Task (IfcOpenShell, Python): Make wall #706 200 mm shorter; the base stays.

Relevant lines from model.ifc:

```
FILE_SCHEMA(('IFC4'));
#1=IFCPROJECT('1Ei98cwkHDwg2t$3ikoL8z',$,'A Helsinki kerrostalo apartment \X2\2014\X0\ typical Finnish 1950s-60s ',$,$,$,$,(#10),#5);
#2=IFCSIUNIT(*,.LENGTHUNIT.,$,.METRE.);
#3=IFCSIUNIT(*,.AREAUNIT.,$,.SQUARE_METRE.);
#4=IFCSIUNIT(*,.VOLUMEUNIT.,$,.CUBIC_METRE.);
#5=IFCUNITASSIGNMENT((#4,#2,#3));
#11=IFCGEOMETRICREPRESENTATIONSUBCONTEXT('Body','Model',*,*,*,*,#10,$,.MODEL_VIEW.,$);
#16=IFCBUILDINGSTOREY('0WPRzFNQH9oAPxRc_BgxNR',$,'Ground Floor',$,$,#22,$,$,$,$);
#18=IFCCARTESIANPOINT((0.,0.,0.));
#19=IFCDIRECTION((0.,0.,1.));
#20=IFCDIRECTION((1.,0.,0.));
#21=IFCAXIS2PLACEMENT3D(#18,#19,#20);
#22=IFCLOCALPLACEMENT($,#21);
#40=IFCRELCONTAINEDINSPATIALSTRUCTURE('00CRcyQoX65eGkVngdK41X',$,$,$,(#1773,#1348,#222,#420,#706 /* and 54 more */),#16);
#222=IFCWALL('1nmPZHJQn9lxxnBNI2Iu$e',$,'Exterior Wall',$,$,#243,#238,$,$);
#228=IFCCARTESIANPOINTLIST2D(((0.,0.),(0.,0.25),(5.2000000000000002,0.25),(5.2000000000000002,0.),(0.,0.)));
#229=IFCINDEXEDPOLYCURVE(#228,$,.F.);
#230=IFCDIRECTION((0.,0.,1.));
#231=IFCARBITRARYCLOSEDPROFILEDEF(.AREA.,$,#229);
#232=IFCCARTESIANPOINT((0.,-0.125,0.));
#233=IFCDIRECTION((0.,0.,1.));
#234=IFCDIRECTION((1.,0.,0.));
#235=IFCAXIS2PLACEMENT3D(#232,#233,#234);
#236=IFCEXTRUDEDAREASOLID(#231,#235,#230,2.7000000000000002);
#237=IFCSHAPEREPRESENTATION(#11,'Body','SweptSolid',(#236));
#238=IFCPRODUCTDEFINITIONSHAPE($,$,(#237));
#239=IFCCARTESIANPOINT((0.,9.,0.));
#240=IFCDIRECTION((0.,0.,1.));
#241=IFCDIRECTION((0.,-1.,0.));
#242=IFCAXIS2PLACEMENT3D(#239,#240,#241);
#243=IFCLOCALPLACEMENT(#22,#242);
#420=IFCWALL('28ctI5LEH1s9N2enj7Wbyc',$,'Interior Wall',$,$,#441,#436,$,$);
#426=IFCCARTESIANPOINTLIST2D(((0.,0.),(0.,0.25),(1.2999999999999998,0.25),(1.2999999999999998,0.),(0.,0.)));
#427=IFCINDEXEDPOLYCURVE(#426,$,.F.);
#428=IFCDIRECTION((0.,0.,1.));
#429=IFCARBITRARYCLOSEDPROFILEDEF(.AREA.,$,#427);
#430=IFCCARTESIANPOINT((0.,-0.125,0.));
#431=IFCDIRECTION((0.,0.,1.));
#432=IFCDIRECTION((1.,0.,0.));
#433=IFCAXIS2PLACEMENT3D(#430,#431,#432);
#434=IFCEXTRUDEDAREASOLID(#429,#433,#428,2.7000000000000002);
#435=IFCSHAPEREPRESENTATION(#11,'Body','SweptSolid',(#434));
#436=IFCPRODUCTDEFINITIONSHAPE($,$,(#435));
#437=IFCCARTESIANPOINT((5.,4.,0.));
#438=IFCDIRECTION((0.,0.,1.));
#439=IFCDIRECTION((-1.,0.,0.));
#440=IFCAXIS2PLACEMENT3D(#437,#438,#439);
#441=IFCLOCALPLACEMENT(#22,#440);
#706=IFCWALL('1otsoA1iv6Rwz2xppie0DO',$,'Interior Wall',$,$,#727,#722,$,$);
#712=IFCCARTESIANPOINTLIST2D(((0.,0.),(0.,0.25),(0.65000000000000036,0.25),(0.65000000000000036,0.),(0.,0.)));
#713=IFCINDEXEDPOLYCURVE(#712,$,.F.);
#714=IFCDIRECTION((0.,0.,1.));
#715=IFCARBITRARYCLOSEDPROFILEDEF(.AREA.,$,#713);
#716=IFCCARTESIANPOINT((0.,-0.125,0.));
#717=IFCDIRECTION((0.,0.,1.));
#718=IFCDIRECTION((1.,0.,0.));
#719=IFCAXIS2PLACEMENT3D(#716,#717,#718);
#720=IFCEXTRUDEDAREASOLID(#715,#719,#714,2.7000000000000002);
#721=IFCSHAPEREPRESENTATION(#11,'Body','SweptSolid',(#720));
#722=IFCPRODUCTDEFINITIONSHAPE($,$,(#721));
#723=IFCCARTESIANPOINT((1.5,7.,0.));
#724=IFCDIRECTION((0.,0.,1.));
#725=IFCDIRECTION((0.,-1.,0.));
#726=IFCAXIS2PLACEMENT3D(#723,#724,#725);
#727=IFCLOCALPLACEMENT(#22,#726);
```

```python
import ifcopenshell
import ifcopenshell.geom
import ifcopenshell.util.representation
import ifcopenshell.util.shape

model = ifcopenshell.open("model.ifc")
settings = ifcopenshell.geom.settings()


def volume(element):
    """Net volume in cubic metres, openings subtracted."""
    shape = ifcopenshell.geom.create_shape(settings, element)
    return ifcopenshell.util.shape.get_volume(shape.geometry)


wall = model.by_id(706)
before = volume(wall)

body = ifcopenshell.util.representation.get_representation(wall, "Model", "Body")
solid = body.Items[0]
old_height = solid.Depth
solid.Depth -= 0.2
after = volume(wall)

print(f"height {old_height:g} -> {solid.Depth:g}, volume {before:.3f} -> {after:.3f} m3")

model.write("model_v2.ifc")
```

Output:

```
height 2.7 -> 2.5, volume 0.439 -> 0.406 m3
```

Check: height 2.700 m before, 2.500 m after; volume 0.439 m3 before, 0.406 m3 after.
